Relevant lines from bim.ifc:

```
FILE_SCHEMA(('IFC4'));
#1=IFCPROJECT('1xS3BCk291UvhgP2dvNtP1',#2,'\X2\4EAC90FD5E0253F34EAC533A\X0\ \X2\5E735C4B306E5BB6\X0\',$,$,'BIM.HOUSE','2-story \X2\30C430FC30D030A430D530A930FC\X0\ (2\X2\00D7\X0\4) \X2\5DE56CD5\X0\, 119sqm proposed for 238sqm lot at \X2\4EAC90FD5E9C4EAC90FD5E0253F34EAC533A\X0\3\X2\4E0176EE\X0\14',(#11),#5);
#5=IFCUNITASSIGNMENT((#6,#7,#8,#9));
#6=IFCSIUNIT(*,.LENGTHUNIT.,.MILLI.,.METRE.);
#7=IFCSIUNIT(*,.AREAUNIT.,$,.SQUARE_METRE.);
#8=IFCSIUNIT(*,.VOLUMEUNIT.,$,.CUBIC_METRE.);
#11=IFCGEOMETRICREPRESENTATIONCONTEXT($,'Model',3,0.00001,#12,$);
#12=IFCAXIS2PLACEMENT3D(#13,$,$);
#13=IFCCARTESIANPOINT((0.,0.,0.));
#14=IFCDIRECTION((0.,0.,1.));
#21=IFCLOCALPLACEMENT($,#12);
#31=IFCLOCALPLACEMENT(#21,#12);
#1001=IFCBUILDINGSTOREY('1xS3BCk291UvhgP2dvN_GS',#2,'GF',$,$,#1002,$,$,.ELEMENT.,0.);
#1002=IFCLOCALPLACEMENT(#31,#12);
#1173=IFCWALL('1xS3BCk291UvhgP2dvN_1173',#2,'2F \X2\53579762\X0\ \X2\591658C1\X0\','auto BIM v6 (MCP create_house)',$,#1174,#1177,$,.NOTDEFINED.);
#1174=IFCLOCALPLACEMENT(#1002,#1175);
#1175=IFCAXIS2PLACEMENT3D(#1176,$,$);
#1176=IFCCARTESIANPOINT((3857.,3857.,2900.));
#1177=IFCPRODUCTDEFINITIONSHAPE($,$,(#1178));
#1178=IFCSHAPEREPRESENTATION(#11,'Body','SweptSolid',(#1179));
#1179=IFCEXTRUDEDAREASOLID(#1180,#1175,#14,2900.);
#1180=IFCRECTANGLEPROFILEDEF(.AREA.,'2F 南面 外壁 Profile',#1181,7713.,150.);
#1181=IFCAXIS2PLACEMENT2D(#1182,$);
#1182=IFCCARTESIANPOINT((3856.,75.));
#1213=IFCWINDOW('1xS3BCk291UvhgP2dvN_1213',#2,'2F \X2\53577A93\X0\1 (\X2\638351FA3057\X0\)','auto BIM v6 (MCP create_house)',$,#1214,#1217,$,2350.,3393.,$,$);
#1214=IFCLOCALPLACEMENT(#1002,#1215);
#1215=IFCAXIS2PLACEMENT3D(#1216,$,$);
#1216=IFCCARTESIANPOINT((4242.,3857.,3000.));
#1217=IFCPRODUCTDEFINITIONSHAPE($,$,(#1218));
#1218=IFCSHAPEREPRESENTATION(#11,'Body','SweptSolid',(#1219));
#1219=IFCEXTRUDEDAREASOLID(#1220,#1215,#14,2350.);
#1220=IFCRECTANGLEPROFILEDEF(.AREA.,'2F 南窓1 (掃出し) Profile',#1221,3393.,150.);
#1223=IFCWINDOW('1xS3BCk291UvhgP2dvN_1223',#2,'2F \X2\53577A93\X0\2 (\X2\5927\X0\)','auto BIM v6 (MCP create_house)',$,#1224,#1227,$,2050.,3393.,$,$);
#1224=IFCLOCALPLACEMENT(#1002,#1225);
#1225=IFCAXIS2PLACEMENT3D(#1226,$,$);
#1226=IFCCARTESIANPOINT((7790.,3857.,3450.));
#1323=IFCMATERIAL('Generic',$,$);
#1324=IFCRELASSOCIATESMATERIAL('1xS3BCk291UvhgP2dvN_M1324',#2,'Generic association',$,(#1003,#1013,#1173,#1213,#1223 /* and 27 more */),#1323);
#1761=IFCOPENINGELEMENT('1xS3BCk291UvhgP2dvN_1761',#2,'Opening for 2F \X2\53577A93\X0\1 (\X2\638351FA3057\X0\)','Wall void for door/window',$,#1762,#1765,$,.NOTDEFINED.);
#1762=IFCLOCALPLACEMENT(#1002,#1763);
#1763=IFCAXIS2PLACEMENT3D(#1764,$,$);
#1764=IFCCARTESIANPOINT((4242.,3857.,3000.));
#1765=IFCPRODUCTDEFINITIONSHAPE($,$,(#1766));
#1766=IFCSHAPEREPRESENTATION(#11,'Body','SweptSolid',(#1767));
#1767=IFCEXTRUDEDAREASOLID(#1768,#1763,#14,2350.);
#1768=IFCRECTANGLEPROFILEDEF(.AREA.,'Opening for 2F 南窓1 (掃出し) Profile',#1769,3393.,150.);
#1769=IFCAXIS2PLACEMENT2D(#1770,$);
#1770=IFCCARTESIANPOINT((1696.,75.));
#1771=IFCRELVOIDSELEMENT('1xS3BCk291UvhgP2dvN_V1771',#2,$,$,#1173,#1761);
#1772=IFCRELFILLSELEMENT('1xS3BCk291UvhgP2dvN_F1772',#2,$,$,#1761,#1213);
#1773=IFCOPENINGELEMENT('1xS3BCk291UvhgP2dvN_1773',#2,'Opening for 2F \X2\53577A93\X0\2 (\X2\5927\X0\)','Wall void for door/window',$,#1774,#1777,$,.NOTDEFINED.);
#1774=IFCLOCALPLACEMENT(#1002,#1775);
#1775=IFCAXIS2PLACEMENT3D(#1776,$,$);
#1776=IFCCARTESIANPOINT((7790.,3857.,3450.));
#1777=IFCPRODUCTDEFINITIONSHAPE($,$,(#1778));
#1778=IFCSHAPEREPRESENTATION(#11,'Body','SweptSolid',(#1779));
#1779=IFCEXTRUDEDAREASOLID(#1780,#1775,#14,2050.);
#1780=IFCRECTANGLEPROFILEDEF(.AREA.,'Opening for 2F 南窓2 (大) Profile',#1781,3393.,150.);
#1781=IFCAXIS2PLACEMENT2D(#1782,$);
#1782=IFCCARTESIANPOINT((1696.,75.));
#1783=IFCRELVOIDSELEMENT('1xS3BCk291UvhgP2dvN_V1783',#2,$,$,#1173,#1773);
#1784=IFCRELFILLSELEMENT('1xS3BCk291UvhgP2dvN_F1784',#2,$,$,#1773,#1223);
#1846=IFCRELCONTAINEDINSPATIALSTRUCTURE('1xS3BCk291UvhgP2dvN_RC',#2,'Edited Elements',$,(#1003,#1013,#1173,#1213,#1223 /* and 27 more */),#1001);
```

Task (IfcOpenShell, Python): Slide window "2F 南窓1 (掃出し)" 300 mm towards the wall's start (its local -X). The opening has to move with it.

```python
import ifcopenshell
import ifcopenshell.api.geometry
import ifcopenshell.util.placement

model = ifcopenshell.open("bim.ifc")

window = model.by_id(1213)
opening = window.FillsVoids[0].RelatingOpeningElement
wall = opening.VoidsElements[0].RelatingBuildingElement

wall_matrix = ifcopenshell.util.placement.get_local_placement(wall.ObjectPlacement)
shift = wall_matrix[:3, 0] * -300.0
before = ifcopenshell.util.placement.get_local_placement(window.ObjectPlacement)[:3, 3].copy()

# The window is not placed relative to its opening, so move both.
for product in (opening, window):
    matrix = ifcopenshell.util.placement.get_local_placement(product.ObjectPlacement)
    matrix[:3, 3] += shift
    ifcopenshell.api.geometry.edit_object_placement(model, product=product, matrix=matrix, is_si=False)

after = ifcopenshell.util.placement.get_local_placement(window.ObjectPlacement)[:3, 3]
print("window moved by", (after - before).round(3) + 0.0)

model.write("bim_rev.ifc")
```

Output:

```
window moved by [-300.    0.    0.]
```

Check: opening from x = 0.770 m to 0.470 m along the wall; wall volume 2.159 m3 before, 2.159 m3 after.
